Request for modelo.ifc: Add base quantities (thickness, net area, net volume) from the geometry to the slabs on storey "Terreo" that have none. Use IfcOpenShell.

First a look at what the model holds.

```python
import ifcopenshell
import ifcopenshell.util.element
import ifcopenshell.util.unit

model = ifcopenshell.open("modelo.ifc")
print(model.schema)
for unit_type in ("LENGTHUNIT", "AREAUNIT", "VOLUMEUNIT"):
    print(unit_type, ifcopenshell.util.unit.calculate_unit_scale(model, unit_type))
storey = next(s for s in model.by_type("IfcBuildingStorey") if s.Name == "Terreo")
slabs = [e for e in ifcopenshell.util.element.get_decomposition(storey) if e.is_a("IfcSlab")]
for e in sorted(slabs, key=lambda e: e.id()):
    print(e.id(), e.is_a(), e.Name, list(ifcopenshell.util.element.get_psets(e, qtos_only=True)), sep=" | ")
```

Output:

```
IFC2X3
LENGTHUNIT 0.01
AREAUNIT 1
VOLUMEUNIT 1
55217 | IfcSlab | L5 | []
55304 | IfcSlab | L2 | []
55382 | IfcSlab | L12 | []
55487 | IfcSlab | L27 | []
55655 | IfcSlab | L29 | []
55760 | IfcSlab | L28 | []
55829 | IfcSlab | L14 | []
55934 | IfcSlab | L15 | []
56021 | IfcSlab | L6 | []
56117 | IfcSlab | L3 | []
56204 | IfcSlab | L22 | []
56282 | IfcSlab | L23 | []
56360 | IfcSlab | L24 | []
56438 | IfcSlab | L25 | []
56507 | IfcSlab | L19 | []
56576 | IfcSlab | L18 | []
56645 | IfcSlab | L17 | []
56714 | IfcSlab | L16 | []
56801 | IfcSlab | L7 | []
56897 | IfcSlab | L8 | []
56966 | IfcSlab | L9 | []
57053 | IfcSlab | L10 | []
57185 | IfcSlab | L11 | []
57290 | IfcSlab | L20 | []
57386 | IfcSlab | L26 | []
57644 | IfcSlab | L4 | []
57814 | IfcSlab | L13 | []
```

```python
import ifcopenshell
import ifcopenshell.api.pset
import ifcopenshell.geom
import ifcopenshell.util.element
import ifcopenshell.util.shape
import ifcopenshell.util.unit

model = ifcopenshell.open("modelo.ifc")
unit_scale = ifcopenshell.util.unit.calculate_unit_scale(model)
area_scale = ifcopenshell.util.unit.calculate_unit_scale(model, "AREAUNIT")
volume_scale = ifcopenshell.util.unit.calculate_unit_scale(model, "VOLUMEUNIT")
settings = ifcopenshell.geom.settings()

storey = next(s for s in model.by_type("IfcBuildingStorey") if s.Name == "Terreo")
slabs = [e for e in ifcopenshell.util.element.get_decomposition(storey) if e.is_a("IfcSlab")]

for e in sorted(slabs, key=lambda e: e.id()):
    if ifcopenshell.util.element.get_psets(e, qtos_only=True, should_inherit=False):
        continue
    # Geometry comes back in metres, in the element's own axes.
    shape = ifcopenshell.geom.create_shape(settings, e)
    values = {
        "Width": ifcopenshell.util.shape.get_z(shape.geometry) / unit_scale,
        "NetArea": ifcopenshell.util.shape.get_footprint_area(shape.geometry) / area_scale,
        "NetVolume": ifcopenshell.util.shape.get_volume(shape.geometry) / volume_scale,
    }
    qto = ifcopenshell.api.pset.add_qto(model, product=e, name="BaseQuantities")
    ifcopenshell.api.pset.edit_qto(model, qto=qto, properties=values)
    print(e.id(), {k: round(v, 3) for k, v in values.items()})

model.write("modelo_edited.ifc")
```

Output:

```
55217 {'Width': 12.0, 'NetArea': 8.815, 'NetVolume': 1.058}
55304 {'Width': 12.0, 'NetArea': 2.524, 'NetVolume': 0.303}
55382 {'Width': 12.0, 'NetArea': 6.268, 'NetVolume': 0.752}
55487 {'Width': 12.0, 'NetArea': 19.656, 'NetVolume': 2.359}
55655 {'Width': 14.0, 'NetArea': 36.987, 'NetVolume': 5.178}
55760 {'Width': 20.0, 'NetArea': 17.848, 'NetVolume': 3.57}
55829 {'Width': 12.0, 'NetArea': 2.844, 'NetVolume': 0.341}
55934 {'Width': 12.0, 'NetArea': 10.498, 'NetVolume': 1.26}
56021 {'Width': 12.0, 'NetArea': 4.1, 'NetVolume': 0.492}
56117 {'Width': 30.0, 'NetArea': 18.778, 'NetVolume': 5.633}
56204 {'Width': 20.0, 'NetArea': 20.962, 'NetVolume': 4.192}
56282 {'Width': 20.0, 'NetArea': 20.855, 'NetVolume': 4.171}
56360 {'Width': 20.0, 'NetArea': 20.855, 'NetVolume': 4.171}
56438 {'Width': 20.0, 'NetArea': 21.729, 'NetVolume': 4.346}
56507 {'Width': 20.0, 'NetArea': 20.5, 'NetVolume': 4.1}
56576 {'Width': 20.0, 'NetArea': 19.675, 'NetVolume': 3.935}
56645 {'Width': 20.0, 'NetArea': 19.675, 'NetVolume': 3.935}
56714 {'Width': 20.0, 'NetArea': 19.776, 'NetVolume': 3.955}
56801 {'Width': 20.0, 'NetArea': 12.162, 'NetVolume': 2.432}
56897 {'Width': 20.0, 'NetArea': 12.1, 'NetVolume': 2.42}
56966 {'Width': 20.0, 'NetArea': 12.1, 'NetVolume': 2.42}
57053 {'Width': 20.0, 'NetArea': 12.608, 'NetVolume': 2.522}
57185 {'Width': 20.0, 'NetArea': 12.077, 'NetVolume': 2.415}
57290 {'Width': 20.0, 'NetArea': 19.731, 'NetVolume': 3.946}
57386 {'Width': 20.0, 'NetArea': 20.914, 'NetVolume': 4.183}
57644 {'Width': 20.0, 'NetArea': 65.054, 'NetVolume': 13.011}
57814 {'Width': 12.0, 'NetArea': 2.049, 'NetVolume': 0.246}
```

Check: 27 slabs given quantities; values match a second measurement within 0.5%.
